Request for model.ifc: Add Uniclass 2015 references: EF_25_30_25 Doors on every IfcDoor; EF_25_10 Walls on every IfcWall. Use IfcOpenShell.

First a look at what the model holds.

```python
import ifcopenshell

model = ifcopenshell.open("model.ifc")
print(model.schema)
print("classifications:", [c.Name for c in model.by_type("IfcClassification")])
for ifc_class in ("IfcDoor", "IfcRoof", "IfcStair", "IfcWall", "IfcWindow"):
    print(ifc_class, len(model.by_type(ifc_class)))
```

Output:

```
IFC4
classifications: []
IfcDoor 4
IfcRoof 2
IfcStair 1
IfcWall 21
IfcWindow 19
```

```python
import ifcopenshell
import ifcopenshell.api.classification

model = ifcopenshell.open("model.ifc")

system = ifcopenshell.api.classification.add_classification(model, classification="Uniclass 2015")

codes = {
    "IfcDoor": ("EF_25_30_25", "Doors"),
    "IfcWall": ("EF_25_10", "Walls"),
}
for ifc_class, (code, name) in codes.items():
    products = model.by_type(ifc_class)
    ifcopenshell.api.classification.add_reference(
        model, products=products, classification=system, identification=code, name=name
    )
    print(code, len(products))

model.write("model_edited.ifc")
```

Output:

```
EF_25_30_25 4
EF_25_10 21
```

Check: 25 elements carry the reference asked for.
